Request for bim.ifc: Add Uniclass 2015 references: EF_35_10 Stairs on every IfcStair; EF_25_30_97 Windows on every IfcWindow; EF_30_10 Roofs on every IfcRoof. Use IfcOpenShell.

First a look at what the model holds.

```python
import ifcopenshell

model = ifcopenshell.open("bim.ifc")
print(model.schema)
print("classifications:", [c.Name for c in model.by_type("IfcClassification")])
for ifc_class in ("IfcDoor", "IfcRoof", "IfcStair", "IfcWall", "IfcWindow"):
    print(ifc_class, len(model.by_type(ifc_class)))
```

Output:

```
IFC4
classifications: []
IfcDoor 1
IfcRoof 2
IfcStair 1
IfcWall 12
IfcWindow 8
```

```python
import ifcopenshell
import ifcopenshell.api.classification

model = ifcopenshell.open("bim.ifc")

system = ifcopenshell.api.classification.add_classification(model, classification="Uniclass 2015")

codes = {
    "IfcStair": ("EF_35_10", "Stairs"),
    "IfcWindow": ("EF_25_30_97", "Windows"),
    "IfcRoof": ("EF_30_10", "Roofs"),
}
for ifc_class, (code, name) in codes.items():
    products = model.by_type(ifc_class)
    ifcopenshell.api.classification.add_reference(
        model, products=products, classification=system, identification=code, name=name
    )
    print(code, len(products))

model.write("bim_edited.ifc")
```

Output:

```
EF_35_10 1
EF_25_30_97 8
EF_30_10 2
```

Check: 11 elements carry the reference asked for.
